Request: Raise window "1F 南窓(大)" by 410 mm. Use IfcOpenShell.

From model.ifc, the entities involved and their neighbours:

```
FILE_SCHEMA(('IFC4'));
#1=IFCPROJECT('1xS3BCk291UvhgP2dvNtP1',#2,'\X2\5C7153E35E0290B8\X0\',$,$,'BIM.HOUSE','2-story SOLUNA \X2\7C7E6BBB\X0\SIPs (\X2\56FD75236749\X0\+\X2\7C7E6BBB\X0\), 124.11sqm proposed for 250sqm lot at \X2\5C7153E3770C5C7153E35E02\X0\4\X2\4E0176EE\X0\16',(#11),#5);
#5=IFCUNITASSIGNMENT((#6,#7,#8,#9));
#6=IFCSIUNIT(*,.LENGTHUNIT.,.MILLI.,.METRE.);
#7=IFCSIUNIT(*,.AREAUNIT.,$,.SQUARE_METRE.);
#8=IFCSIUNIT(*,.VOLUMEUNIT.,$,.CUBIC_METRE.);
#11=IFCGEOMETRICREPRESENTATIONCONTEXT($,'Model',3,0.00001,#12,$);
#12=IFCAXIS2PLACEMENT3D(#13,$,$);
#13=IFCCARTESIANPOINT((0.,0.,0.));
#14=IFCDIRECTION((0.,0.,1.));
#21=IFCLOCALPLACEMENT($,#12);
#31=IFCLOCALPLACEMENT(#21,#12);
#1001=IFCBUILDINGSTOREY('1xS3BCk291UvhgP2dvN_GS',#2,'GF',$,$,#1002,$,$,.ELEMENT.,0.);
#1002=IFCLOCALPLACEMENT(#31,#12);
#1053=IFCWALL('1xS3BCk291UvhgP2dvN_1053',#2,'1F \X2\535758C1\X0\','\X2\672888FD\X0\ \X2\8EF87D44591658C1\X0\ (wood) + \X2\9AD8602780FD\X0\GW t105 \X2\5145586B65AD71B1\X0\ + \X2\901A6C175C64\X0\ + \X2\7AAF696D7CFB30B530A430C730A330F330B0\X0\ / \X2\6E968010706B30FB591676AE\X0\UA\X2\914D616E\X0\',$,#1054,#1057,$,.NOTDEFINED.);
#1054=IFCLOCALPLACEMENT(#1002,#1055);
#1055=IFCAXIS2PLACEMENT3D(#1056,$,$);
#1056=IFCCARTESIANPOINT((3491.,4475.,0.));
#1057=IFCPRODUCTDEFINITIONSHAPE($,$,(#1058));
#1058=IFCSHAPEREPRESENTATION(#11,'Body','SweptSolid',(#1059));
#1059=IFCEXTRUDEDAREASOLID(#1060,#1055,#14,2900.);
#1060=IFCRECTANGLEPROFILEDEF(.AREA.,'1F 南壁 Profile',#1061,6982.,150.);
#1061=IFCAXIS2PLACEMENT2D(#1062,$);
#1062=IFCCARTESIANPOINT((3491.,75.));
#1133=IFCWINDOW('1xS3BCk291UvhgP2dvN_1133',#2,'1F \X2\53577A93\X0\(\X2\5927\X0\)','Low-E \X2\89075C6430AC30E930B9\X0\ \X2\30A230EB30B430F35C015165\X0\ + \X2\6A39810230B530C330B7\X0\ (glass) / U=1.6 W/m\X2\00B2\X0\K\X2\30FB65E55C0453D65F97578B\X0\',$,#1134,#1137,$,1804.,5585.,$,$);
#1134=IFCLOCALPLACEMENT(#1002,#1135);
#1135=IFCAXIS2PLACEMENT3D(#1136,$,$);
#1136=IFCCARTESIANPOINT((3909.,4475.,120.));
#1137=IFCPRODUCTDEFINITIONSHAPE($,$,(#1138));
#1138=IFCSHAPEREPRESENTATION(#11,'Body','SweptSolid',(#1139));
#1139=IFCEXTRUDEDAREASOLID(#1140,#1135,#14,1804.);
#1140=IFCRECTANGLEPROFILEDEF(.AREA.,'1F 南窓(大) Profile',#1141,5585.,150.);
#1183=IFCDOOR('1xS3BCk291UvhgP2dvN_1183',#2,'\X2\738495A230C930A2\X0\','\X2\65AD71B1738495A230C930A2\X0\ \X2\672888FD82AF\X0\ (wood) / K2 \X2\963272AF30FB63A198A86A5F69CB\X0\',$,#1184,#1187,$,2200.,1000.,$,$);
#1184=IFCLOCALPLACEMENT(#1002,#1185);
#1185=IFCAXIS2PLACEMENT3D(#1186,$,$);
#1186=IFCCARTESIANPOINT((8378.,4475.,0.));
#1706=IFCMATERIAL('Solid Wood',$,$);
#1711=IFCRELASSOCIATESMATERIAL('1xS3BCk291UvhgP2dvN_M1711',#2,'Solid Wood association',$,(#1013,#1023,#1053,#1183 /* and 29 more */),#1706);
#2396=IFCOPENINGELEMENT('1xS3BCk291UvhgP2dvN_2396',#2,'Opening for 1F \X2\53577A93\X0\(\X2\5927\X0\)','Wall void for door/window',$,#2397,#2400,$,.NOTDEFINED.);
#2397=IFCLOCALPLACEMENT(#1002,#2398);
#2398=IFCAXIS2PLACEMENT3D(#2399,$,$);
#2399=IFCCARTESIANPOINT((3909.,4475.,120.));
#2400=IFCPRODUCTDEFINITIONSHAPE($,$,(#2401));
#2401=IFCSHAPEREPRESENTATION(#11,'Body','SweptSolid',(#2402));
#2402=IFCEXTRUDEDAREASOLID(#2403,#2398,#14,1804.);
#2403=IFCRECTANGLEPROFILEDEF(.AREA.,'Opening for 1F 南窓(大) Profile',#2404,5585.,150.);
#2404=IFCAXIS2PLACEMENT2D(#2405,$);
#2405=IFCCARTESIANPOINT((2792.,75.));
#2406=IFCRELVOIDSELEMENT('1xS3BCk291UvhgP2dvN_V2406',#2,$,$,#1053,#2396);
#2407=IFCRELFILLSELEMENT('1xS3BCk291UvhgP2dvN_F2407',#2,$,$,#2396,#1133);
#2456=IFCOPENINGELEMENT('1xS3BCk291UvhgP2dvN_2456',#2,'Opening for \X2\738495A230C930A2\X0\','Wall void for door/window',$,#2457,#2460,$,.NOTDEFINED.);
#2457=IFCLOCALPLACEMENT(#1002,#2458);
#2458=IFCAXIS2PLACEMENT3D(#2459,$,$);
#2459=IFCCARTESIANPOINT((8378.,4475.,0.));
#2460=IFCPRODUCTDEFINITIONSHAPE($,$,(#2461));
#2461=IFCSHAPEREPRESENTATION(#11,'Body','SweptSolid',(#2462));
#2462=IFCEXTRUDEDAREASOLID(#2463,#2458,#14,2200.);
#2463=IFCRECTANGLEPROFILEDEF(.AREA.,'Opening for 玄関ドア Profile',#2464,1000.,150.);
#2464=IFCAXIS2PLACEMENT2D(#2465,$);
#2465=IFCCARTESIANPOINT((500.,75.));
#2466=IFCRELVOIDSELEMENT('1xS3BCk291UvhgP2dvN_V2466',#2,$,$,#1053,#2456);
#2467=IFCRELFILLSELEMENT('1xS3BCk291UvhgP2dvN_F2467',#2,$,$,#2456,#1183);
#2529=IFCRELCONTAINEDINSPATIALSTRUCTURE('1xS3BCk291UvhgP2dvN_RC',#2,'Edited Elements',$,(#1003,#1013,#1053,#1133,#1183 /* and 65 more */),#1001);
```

```python
import numpy as np
import ifcopenshell
import ifcopenshell.api.geometry
import ifcopenshell.util.placement
import ifcopenshell.util.unit

model = ifcopenshell.open("model.ifc")
unit_scale = ifcopenshell.util.unit.calculate_unit_scale(model)

window = model.by_guid("1xS3BCk291UvhgP2dvN_1133")
opening = window.FillsVoids[0].RelatingOpeningElement
dz = 0.41 / unit_scale

shift = np.array([0.0, 0.0, dz])
# The window is not placed relative to its opening, so move both.
for product in (opening, window):
    matrix = ifcopenshell.util.placement.get_local_placement(product.ObjectPlacement)
    matrix[:3, 3] += shift
    ifcopenshell.api.geometry.edit_object_placement(model, product=product, matrix=matrix, is_si=False)

print(f"moved by {dz * unit_scale:+.3f} m")

model.write("model_v2.ifc")
```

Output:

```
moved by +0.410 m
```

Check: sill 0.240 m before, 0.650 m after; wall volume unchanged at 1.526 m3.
